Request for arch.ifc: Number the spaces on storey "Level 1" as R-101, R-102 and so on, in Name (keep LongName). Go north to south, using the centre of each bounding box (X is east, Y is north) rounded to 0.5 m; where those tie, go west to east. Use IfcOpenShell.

First a look at what the model holds.

```python
import ifcopenshell
import ifcopenshell.util.element
import ifcopenshell.util.placement

model = ifcopenshell.open("arch.ifc")
print(model.schema)
storey = next(s for s in model.by_type("IfcBuildingStorey") if s.Name == "Level 1")
spaces = [e for e in ifcopenshell.util.element.get_decomposition(storey) if e.is_a("IfcSpace")]
for e in sorted(spaces, key=lambda e: e.id()):
    origin = ifcopenshell.util.placement.get_local_placement(e.ObjectPlacement)[:3, 3]
    print(e.id(), e.Name, e.LongName, origin.round(2) + 0.0, sep=" | ")
```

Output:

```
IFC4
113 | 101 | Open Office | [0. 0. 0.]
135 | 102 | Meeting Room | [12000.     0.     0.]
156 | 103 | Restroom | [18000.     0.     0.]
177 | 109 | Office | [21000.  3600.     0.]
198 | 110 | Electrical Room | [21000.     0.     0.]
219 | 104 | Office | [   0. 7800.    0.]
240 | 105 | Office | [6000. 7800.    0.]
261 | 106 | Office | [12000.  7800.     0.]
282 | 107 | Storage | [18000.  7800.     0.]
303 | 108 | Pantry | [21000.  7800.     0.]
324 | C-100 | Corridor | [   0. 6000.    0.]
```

```python
import ifcopenshell
import ifcopenshell.geom
import ifcopenshell.util.element
import ifcopenshell.util.shape

model = ifcopenshell.open("arch.ifc")
settings = ifcopenshell.geom.settings()
settings.set("use-world-coords", True)


def centre(element):
    shape = ifcopenshell.geom.create_shape(settings, element)
    return ifcopenshell.util.shape.get_bbox_centroid(shape.geometry)


storey = next(s for s in model.by_type("IfcBuildingStorey") if s.Name == "Level 1")
spaces = [e for e in ifcopenshell.util.element.get_decomposition(storey) if e.is_a("IfcSpace")]

# Insertion points can sit at a corner or the storey origin, so sort by the geometry (in metres).
centres = {e: centre(e) for e in spaces}
spaces.sort(key=lambda e: (-round(centres[e][1] / 0.5), centres[e][0]))

for i, e in enumerate(spaces, start=1):
    number = f"R-1{i:02d}"
    e.Name = number
    print(e.id(), number)

model.write("arch_edited.ifc")
```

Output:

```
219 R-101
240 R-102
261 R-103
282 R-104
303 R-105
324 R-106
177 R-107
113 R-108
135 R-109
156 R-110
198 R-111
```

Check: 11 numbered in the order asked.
